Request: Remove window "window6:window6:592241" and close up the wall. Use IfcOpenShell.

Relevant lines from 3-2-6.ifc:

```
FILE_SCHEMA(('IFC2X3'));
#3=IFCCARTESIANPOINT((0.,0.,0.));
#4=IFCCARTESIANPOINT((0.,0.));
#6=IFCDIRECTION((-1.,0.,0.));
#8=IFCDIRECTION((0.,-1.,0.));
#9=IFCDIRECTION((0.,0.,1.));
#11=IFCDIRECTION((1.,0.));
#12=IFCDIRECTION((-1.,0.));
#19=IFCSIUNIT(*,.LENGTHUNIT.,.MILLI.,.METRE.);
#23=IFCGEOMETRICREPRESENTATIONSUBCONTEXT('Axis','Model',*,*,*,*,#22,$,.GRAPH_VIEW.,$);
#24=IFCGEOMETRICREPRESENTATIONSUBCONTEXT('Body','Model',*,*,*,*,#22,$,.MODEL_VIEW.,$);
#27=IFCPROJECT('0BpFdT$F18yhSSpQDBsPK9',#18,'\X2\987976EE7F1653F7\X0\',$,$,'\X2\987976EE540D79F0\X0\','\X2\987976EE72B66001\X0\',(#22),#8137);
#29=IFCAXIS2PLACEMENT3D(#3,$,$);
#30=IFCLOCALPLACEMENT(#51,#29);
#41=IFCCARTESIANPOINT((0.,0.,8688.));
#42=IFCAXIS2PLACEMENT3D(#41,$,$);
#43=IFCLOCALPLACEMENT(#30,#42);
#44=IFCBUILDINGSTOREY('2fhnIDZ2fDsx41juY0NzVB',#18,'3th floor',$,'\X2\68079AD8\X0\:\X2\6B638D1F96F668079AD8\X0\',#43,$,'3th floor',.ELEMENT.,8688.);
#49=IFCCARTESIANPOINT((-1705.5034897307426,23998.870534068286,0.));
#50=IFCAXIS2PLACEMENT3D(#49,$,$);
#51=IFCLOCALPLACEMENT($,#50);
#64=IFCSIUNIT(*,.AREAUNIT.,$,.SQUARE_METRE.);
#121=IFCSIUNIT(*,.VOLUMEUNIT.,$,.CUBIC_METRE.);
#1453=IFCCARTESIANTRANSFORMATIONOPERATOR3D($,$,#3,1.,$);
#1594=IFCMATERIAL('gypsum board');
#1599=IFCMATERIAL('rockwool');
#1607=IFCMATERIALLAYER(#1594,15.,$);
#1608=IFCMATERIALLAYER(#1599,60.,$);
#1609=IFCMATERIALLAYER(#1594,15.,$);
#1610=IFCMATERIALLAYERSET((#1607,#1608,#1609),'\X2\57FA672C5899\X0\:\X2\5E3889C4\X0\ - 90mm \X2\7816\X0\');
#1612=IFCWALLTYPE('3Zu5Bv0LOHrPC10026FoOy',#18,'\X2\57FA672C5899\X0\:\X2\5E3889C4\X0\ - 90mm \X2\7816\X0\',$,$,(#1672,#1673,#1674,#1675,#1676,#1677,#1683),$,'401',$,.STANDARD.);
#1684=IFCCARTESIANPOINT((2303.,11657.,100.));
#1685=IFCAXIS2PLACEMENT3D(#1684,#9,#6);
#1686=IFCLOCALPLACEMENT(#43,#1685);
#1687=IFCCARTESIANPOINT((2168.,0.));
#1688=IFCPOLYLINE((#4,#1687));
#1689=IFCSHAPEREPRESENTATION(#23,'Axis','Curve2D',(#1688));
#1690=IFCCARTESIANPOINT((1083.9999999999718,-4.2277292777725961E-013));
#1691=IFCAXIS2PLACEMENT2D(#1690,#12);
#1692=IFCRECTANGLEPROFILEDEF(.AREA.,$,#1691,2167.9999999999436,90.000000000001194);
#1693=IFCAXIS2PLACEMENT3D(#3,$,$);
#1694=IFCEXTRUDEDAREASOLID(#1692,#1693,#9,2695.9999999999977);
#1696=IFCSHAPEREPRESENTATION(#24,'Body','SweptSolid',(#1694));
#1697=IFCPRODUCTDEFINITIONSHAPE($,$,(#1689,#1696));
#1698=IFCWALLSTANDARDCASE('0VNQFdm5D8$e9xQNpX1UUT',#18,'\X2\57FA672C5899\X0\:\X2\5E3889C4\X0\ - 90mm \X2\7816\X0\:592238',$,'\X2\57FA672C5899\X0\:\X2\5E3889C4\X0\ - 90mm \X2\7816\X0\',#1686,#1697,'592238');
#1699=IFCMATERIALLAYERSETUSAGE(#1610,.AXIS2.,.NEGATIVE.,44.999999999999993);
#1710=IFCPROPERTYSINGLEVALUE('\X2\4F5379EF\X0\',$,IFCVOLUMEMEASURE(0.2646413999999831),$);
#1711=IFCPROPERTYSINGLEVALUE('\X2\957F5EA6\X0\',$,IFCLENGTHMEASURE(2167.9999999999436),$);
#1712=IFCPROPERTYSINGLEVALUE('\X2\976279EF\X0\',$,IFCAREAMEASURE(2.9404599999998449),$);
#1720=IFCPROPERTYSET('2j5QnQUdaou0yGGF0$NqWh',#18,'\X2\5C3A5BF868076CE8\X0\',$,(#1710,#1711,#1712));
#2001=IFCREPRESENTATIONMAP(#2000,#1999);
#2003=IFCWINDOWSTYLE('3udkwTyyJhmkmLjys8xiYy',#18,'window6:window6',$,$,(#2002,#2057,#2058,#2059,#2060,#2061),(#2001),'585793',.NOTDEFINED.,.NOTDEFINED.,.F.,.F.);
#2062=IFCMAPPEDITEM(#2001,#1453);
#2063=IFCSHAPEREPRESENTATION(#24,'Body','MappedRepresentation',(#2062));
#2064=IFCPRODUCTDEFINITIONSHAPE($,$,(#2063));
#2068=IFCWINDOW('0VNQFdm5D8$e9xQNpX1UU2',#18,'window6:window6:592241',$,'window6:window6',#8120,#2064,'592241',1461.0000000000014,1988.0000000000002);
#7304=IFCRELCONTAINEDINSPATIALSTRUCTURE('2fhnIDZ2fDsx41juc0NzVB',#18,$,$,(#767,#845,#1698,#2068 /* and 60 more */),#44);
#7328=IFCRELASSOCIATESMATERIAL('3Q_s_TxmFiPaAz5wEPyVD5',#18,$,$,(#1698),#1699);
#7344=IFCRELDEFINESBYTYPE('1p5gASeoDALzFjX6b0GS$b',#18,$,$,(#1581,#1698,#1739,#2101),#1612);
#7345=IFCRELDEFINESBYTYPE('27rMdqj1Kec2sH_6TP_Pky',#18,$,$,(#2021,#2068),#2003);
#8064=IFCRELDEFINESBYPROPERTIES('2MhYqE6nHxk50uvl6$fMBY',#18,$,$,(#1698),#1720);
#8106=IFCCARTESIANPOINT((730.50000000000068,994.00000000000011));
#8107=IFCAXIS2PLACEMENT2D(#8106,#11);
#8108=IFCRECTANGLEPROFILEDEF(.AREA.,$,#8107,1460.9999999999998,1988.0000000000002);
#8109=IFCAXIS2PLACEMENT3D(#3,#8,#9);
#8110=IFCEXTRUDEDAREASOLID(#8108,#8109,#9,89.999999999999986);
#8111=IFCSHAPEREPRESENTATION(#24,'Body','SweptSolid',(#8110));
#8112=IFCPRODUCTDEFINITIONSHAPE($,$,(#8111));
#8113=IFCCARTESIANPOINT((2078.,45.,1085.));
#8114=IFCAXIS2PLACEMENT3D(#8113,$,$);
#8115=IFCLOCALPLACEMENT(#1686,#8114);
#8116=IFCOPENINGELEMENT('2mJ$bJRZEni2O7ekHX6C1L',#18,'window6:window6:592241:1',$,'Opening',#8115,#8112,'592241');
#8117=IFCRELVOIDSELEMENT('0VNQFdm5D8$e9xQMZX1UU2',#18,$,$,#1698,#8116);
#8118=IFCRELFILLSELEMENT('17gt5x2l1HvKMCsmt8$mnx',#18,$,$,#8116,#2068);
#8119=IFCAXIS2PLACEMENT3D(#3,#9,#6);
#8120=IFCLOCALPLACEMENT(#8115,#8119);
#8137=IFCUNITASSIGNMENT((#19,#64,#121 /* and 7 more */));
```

```python
import ifcopenshell
import ifcopenshell.api.feature
import ifcopenshell.api.pset
import ifcopenshell.api.root
import ifcopenshell.geom
import ifcopenshell.util.element
import ifcopenshell.util.shape
import ifcopenshell.util.unit

model = ifcopenshell.open("3-2-6.ifc")
area_scale = ifcopenshell.util.unit.calculate_unit_scale(model, "AREAUNIT")
volume_scale = ifcopenshell.util.unit.calculate_unit_scale(model, "VOLUMEUNIT")
settings = ifcopenshell.geom.settings()


def volume(element):
    """Net volume in cubic metres, openings subtracted."""
    shape = ifcopenshell.geom.create_shape(settings, element)
    return ifcopenshell.util.shape.get_volume(shape.geometry)


window = model.by_id(2068)
opening = window.FillsVoids[0].RelatingOpeningElement
wall = opening.VoidsElements[0].RelatingBuildingElement
before = volume(wall)

ifcopenshell.api.root.remove_product(model, product=window)
ifcopenshell.api.feature.remove_feature(model, feature=opening)

after = volume(wall)
thickness = 0.09  # wall thickness in metres

# Update the wall's stored quantities.
pset = model.by_id(ifcopenshell.util.element.get_pset(wall, "尺寸标注", should_inherit=False)["id"])
ifcopenshell.api.pset.edit_pset(model, pset=pset, properties={
    "体积": model.create_entity("IfcVolumeMeasure", after / volume_scale),
    "面积": model.create_entity("IfcAreaMeasure", after / thickness / area_scale),
})

print(f"wall volume {before:.3f} -> {after:.3f} m3")

model.write("3-2-6-out.ifc")
```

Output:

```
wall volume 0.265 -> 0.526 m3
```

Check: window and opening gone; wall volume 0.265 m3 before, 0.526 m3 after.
